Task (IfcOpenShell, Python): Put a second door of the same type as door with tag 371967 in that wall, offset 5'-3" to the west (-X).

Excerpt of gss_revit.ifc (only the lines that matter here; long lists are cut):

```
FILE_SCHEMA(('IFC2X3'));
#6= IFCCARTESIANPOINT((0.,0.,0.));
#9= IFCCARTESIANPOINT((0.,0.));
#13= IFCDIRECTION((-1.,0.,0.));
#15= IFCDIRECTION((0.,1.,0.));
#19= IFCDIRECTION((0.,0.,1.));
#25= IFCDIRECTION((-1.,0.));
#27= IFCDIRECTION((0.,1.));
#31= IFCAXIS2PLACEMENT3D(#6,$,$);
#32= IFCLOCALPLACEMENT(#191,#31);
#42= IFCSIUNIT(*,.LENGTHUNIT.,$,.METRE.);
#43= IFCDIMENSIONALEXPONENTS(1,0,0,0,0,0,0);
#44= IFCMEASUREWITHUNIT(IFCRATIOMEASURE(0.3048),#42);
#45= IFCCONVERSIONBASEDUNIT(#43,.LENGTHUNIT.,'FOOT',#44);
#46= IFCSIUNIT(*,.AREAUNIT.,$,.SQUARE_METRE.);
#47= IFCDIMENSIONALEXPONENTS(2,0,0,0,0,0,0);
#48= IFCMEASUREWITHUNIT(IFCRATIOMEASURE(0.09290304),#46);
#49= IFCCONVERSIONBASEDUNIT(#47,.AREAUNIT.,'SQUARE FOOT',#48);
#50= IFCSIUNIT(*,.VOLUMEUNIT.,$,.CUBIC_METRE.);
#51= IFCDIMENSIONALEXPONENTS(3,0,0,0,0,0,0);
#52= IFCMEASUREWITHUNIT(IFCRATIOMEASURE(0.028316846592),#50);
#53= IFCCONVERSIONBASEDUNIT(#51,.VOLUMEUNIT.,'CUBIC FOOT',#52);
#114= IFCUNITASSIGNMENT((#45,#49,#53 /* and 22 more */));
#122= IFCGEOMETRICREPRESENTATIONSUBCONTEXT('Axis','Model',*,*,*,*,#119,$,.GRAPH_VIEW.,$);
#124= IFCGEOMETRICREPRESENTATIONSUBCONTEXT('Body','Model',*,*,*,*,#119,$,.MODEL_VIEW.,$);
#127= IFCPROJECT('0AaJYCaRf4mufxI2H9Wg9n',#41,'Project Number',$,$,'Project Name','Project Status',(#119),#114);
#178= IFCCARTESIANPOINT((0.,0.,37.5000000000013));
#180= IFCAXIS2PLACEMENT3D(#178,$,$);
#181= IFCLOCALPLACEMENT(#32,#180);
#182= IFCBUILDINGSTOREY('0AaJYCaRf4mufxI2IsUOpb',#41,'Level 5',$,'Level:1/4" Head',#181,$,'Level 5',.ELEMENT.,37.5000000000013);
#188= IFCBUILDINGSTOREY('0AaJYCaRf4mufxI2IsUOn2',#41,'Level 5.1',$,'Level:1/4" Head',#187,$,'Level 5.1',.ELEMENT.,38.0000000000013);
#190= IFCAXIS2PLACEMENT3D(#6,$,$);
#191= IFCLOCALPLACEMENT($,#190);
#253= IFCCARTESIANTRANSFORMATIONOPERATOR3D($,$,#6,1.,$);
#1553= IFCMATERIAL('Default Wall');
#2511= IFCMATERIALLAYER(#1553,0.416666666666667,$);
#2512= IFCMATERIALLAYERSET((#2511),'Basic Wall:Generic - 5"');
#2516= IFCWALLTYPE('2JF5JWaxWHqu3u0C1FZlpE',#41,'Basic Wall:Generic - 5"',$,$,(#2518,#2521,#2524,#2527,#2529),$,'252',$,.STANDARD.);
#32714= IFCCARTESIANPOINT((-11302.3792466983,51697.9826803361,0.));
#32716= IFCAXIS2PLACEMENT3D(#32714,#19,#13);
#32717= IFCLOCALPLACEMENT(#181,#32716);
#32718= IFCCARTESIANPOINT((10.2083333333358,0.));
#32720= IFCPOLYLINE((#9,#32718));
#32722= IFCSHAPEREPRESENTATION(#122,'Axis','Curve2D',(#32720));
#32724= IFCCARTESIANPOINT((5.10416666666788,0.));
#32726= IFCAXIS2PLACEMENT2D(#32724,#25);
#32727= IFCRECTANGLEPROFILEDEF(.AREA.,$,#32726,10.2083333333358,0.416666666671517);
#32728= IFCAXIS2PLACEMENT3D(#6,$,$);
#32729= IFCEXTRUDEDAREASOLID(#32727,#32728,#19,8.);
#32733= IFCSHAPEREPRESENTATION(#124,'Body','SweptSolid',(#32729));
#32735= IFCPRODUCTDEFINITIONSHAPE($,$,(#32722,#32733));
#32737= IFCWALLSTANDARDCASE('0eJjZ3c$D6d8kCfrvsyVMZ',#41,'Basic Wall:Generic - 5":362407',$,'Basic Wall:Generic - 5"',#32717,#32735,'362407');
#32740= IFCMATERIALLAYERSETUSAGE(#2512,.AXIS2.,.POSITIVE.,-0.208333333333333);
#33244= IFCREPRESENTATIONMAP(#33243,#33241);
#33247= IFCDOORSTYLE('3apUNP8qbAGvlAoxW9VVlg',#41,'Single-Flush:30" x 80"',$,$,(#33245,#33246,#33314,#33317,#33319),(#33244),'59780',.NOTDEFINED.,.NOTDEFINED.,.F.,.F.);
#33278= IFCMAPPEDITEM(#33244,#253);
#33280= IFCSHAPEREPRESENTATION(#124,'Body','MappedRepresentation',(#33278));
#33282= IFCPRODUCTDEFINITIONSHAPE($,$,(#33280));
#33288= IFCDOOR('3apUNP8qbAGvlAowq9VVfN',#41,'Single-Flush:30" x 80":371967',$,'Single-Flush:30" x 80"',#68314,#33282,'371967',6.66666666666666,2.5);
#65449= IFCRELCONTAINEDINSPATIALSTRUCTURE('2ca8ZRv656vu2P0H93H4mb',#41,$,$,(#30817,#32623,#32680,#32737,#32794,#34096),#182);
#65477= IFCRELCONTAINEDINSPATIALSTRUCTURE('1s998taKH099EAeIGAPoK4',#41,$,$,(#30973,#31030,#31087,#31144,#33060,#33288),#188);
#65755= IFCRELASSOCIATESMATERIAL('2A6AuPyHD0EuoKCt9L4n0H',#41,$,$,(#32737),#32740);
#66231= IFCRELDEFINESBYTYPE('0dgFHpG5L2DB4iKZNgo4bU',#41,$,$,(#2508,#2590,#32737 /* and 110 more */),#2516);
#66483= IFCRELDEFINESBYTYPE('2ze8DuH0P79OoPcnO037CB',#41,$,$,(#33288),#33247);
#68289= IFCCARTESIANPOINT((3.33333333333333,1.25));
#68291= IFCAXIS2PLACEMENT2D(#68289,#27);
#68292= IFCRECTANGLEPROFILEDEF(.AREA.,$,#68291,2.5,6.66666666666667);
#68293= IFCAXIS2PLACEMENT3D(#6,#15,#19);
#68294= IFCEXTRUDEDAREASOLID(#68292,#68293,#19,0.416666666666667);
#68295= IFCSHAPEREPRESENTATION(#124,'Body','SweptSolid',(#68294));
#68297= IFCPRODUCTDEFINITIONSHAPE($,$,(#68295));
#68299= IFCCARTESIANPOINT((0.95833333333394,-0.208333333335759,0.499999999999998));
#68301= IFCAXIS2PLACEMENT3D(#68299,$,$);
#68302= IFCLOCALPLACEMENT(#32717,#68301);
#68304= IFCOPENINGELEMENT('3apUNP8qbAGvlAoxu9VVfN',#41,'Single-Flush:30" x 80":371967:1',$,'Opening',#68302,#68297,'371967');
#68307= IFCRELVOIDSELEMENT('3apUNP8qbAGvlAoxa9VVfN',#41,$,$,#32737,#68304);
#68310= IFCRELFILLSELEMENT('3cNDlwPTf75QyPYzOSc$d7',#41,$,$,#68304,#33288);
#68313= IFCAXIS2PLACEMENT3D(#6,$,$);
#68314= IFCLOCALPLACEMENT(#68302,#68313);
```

```python
import ifcopenshell
import ifcopenshell.api.feature
import ifcopenshell.api.geometry
import ifcopenshell.api.root
import ifcopenshell.geom
import ifcopenshell.util.element
import ifcopenshell.util.placement
import ifcopenshell.util.shape
import ifcopenshell.util.unit

model = ifcopenshell.open("gss_revit.ifc")
unit_scale = ifcopenshell.util.unit.calculate_unit_scale(model)
settings = ifcopenshell.geom.settings()


def volume(element):
    """Net volume in cubic metres, openings subtracted."""
    shape = ifcopenshell.geom.create_shape(settings, element)
    return ifcopenshell.util.shape.get_volume(shape.geometry)


def reuse_history(source, copy):
    """copy_class also copies each property set's owner history, people and application; keep the originals."""
    for rel in copy.IsDefinedBy:
        if rel.is_a("IfcRelDefinesByProperties") and (history := rel.RelatingPropertyDefinition.OwnerHistory):
            rel.RelatingPropertyDefinition.OwnerHistory = source.OwnerHistory
            ifcopenshell.util.element.remove_deep2(model, history)


door = model.by_guid("3apUNP8qbAGvlAowq9VVfN")
opening = door.FillsVoids[0].RelatingOpeningElement
wall = opening.VoidsElements[0].RelatingBuildingElement
before = volume(wall)
shift = ifcopenshell.util.placement.get_local_placement(wall.ObjectPlacement)[:3, 0] * 63 * 0.0254 / unit_scale

# copy_class copies the void relationship, type, container and properties, but no geometry.
new_opening = ifcopenshell.api.root.copy_class(model, product=opening)
new_opening.Representation = ifcopenshell.util.element.copy_deep(
    model, opening.Representation, exclude=["IfcGeometricRepresentationContext", "IfcRepresentationMap"]
)
new_opening.Name = 'Single-Flush:30" x 80"'
new_opening.Tag = None
new_door = ifcopenshell.api.root.copy_class(model, product=door)
new_door.Representation = ifcopenshell.util.element.copy_deep(
    model, door.Representation, exclude=["IfcGeometricRepresentationContext", "IfcRepresentationMap"]
)
new_door.Name = 'Single-Flush:30" x 80"'
new_door.Tag = None
reuse_history(door, new_door)
fills = ifcopenshell.api.feature.add_filling(model, opening=new_opening, element=new_door)
fills.OwnerHistory = new_door.OwnerHistory  # required in IFC2X3

for old, new in ((opening, new_opening), (door, new_door)):
    matrix = ifcopenshell.util.placement.get_local_placement(old.ObjectPlacement)
    matrix[:3, 3] += shift
    ifcopenshell.api.geometry.edit_object_placement(model, product=new, matrix=matrix, is_si=False)

after = volume(wall)

print(f"wall volume {before:.3f} -> {after:.3f} m3")

model.write("gss_revit_rev.ifc")
```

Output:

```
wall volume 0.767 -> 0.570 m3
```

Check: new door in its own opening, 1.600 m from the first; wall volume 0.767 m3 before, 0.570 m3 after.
